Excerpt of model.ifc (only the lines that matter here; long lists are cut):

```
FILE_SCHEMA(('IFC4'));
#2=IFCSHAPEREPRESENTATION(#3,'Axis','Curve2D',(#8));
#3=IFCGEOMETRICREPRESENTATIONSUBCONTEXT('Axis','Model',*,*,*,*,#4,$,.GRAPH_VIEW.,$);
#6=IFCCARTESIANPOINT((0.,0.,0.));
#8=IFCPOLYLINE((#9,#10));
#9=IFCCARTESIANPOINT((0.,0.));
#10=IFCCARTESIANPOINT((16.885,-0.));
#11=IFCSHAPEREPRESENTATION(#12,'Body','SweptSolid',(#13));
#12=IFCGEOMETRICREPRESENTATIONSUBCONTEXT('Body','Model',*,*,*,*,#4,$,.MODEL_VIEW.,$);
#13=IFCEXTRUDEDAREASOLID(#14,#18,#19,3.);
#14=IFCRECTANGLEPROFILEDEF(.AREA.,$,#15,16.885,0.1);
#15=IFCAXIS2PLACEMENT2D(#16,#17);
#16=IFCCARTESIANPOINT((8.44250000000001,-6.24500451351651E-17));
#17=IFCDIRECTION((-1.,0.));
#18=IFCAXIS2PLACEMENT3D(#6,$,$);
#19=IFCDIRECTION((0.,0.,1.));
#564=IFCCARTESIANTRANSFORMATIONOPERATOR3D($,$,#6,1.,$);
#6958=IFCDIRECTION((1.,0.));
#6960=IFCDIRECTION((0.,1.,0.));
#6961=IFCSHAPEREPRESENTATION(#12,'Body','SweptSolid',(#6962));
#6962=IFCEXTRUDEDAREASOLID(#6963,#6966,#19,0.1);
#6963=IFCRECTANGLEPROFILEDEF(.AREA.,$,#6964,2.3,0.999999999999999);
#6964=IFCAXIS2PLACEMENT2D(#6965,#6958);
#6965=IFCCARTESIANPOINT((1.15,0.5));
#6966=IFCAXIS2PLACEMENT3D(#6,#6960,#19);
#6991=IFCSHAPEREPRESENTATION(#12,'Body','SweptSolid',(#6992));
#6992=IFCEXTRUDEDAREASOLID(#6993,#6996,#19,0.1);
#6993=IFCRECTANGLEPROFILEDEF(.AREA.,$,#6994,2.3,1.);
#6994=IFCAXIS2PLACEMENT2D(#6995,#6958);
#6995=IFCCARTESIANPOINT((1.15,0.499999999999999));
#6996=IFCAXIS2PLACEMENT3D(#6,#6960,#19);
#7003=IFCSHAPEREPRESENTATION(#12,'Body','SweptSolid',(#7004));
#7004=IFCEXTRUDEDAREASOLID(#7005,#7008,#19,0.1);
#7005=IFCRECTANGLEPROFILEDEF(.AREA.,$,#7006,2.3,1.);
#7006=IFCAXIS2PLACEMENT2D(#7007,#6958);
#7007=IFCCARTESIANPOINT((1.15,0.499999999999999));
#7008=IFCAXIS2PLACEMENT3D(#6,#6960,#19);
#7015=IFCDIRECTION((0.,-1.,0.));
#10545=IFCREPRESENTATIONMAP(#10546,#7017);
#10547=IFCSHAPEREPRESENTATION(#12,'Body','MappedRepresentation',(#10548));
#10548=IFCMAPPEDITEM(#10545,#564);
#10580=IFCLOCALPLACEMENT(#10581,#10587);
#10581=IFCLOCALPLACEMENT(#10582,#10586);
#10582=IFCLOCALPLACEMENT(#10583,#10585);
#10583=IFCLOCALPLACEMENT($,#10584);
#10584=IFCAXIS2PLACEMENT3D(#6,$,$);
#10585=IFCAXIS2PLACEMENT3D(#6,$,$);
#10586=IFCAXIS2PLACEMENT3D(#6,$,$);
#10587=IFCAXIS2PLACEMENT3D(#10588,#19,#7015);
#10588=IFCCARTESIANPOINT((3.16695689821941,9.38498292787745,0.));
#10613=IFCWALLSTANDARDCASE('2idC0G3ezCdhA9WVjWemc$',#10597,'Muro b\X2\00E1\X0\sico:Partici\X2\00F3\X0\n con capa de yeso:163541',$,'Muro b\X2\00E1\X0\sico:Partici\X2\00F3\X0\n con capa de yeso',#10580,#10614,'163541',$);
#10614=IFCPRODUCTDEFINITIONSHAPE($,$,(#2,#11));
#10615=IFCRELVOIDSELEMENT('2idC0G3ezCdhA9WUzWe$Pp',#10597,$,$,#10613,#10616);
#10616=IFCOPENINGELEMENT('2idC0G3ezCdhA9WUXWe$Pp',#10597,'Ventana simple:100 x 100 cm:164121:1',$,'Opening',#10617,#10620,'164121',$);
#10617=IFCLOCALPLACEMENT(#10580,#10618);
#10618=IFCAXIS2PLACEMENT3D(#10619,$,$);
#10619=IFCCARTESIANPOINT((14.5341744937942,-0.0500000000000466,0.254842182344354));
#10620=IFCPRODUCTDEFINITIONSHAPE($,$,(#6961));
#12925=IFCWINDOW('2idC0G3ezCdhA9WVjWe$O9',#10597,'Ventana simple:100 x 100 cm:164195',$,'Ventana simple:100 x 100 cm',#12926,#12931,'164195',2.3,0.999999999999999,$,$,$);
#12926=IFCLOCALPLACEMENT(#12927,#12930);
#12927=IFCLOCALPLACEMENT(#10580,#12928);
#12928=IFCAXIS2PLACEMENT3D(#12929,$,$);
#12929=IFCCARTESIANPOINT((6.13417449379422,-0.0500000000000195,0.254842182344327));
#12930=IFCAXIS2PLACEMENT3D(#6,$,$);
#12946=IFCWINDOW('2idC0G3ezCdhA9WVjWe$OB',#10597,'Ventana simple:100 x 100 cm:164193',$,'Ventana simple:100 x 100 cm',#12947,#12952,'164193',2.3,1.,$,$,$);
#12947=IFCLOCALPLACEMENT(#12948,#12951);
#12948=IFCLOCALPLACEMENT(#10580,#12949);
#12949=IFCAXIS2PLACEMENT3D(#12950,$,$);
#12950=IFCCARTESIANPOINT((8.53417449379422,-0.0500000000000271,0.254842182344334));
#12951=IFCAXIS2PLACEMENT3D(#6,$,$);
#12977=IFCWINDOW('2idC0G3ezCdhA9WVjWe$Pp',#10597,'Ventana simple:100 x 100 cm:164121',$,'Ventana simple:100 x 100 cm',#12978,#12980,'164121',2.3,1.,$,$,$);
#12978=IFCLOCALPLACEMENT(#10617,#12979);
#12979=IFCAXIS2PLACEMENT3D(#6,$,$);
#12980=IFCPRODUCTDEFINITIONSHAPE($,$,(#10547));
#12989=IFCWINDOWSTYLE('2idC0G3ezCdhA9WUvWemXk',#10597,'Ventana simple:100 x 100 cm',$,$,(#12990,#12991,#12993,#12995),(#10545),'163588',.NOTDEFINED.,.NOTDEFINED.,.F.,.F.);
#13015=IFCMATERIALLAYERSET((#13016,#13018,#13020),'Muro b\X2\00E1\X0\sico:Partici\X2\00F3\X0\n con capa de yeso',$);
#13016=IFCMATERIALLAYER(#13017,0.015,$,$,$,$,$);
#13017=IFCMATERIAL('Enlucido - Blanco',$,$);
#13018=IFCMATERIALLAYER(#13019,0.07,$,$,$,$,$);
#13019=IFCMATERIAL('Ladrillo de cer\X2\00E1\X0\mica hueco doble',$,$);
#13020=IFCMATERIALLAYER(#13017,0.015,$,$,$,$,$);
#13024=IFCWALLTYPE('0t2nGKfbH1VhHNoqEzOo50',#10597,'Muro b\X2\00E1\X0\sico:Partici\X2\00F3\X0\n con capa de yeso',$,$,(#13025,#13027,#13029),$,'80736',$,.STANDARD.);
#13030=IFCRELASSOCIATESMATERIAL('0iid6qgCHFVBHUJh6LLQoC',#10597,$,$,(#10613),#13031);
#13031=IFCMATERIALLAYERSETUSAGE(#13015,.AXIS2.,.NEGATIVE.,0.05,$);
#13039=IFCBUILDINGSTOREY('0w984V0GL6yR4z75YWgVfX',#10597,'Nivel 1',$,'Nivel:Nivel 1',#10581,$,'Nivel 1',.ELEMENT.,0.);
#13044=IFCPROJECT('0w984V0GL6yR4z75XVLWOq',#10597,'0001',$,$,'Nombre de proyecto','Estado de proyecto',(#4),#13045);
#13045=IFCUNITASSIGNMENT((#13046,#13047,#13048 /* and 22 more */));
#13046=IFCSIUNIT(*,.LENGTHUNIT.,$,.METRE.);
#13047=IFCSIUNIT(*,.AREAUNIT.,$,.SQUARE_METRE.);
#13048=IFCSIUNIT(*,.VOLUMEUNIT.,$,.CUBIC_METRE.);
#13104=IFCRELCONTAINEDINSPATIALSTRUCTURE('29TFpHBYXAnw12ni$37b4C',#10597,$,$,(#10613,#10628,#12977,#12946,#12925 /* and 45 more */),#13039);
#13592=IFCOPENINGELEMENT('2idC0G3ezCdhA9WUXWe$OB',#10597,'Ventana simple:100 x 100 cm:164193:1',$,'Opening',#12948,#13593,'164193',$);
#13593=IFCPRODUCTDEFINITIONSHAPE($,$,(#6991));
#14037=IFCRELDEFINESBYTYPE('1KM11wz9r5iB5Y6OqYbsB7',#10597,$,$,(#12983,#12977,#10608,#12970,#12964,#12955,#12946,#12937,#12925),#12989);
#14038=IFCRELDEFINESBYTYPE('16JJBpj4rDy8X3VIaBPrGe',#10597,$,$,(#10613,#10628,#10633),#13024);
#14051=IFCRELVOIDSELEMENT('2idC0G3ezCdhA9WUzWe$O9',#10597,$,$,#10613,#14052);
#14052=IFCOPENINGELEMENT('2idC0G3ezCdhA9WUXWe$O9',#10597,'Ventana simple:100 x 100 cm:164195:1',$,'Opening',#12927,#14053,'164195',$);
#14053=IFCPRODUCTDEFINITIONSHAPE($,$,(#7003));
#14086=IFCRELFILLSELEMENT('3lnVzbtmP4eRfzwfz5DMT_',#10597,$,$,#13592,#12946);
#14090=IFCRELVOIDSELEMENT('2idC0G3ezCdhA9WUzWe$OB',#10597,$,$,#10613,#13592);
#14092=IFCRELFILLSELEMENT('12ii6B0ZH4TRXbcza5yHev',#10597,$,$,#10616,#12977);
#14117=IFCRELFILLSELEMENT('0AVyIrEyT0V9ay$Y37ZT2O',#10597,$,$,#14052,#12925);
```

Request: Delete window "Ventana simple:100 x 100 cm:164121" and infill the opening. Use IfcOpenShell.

```python
import ifcopenshell
import ifcopenshell.api.feature
import ifcopenshell.api.root
import ifcopenshell.geom
import ifcopenshell.util.shape

model = ifcopenshell.open("model.ifc")
settings = ifcopenshell.geom.settings()


def volume(element):
    """Net volume in cubic metres, openings subtracted."""
    shape = ifcopenshell.geom.create_shape(settings, element)
    return ifcopenshell.util.shape.get_volume(shape.geometry)


window = model.by_id(12977)
opening = window.FillsVoids[0].RelatingOpeningElement
wall = opening.VoidsElements[0].RelatingBuildingElement
before = volume(wall)

ifcopenshell.api.root.remove_product(model, product=window)
ifcopenshell.api.feature.remove_feature(model, feature=opening)

after = volume(wall)

print(f"wall volume {before:.3f} -> {after:.3f} m3")

model.write("model_updated.ifc")
```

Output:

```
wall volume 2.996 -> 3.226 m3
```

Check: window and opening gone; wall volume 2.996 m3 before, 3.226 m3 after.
